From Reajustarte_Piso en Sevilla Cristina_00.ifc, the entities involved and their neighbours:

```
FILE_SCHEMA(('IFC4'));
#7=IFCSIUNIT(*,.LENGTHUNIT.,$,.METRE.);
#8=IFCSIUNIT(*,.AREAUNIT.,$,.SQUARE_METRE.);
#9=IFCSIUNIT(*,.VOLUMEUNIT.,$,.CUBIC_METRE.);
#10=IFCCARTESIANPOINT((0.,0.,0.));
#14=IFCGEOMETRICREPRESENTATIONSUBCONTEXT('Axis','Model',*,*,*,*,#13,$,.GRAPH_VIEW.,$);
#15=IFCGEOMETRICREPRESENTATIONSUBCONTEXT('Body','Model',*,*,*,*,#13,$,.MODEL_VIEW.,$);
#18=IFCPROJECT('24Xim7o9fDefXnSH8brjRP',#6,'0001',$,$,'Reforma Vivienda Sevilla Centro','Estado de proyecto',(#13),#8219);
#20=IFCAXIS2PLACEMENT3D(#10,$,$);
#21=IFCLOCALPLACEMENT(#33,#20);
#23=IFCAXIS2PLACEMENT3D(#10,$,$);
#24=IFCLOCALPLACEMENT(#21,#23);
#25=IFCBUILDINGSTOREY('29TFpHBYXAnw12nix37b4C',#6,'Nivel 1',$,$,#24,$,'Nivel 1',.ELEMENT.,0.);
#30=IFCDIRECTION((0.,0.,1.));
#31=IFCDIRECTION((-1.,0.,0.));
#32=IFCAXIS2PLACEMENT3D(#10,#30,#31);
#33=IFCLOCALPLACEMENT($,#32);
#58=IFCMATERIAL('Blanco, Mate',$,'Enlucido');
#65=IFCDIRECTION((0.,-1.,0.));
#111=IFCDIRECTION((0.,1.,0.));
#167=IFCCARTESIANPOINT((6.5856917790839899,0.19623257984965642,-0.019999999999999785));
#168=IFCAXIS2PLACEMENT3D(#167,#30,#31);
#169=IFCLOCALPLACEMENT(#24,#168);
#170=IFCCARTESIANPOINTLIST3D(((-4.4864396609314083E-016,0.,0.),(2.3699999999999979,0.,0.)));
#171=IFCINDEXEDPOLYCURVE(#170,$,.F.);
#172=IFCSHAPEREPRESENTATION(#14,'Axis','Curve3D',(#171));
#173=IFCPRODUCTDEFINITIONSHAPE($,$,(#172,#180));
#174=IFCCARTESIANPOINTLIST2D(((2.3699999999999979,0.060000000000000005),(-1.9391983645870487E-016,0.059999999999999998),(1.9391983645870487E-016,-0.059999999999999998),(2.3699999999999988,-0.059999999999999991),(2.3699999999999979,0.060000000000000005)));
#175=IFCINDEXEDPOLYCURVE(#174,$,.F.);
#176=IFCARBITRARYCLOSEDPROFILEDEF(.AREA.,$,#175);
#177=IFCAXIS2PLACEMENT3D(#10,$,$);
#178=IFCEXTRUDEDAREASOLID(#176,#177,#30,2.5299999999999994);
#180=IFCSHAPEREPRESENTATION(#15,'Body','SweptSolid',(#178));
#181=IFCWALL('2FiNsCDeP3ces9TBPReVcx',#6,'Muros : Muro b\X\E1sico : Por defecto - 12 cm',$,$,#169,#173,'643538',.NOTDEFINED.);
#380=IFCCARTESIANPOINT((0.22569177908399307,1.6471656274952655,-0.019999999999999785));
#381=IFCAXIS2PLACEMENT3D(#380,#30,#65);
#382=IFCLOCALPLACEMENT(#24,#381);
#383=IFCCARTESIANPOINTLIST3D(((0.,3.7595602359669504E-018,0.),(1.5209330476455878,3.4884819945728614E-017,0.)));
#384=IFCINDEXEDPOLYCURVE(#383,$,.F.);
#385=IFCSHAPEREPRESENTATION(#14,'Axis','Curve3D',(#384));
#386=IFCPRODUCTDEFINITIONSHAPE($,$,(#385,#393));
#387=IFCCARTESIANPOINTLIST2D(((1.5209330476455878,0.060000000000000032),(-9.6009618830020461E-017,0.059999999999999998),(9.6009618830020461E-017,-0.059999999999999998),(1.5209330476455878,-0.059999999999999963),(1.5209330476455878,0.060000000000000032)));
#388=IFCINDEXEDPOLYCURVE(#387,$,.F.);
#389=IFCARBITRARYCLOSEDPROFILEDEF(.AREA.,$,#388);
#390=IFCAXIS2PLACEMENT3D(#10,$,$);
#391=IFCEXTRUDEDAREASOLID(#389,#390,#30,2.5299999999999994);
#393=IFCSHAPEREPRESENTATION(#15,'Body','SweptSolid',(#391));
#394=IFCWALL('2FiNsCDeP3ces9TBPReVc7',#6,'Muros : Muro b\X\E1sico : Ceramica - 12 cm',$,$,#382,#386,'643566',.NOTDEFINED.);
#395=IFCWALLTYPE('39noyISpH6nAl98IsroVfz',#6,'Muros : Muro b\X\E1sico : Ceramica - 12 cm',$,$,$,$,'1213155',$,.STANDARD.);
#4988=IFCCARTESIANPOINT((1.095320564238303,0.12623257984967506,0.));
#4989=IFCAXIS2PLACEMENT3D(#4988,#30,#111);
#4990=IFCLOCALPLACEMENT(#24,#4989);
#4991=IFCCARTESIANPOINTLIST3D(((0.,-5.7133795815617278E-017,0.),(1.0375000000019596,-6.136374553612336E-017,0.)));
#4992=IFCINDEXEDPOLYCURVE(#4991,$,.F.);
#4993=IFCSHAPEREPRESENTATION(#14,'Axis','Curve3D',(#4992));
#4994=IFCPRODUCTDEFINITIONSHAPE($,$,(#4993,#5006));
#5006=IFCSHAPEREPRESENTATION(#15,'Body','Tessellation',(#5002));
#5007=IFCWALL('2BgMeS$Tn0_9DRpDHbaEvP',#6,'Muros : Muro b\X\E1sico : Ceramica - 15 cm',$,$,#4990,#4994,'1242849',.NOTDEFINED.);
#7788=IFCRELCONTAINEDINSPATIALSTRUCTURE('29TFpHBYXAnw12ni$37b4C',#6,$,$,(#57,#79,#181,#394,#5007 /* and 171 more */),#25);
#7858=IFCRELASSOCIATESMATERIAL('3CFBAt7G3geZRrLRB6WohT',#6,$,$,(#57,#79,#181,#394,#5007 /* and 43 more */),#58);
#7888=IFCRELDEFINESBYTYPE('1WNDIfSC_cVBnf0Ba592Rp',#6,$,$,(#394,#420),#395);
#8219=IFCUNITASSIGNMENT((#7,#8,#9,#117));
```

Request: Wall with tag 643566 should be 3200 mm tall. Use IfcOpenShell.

```python
import ifcopenshell
import ifcopenshell.geom
import ifcopenshell.util.representation
import ifcopenshell.util.shape

model = ifcopenshell.open("Reajustarte_Piso en Sevilla Cristina_00.ifc")
settings = ifcopenshell.geom.settings()


def volume(element):
    """Net volume in cubic metres, openings subtracted."""
    shape = ifcopenshell.geom.create_shape(settings, element)
    return ifcopenshell.util.shape.get_volume(shape.geometry)


wall = model.by_id(394)
before = volume(wall)

body = ifcopenshell.util.representation.get_representation(wall, "Model", "Body")
solid = body.Items[0]
old_height = solid.Depth
solid.Depth = 3.2
after = volume(wall)

print(f"height {old_height:g} -> {solid.Depth:g}, volume {before:.3f} -> {after:.3f} m3")

model.write("Reajustarte_Piso en Sevilla Cristina_00-out.ifc")
```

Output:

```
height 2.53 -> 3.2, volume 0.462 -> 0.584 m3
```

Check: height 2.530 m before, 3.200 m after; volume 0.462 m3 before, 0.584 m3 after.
